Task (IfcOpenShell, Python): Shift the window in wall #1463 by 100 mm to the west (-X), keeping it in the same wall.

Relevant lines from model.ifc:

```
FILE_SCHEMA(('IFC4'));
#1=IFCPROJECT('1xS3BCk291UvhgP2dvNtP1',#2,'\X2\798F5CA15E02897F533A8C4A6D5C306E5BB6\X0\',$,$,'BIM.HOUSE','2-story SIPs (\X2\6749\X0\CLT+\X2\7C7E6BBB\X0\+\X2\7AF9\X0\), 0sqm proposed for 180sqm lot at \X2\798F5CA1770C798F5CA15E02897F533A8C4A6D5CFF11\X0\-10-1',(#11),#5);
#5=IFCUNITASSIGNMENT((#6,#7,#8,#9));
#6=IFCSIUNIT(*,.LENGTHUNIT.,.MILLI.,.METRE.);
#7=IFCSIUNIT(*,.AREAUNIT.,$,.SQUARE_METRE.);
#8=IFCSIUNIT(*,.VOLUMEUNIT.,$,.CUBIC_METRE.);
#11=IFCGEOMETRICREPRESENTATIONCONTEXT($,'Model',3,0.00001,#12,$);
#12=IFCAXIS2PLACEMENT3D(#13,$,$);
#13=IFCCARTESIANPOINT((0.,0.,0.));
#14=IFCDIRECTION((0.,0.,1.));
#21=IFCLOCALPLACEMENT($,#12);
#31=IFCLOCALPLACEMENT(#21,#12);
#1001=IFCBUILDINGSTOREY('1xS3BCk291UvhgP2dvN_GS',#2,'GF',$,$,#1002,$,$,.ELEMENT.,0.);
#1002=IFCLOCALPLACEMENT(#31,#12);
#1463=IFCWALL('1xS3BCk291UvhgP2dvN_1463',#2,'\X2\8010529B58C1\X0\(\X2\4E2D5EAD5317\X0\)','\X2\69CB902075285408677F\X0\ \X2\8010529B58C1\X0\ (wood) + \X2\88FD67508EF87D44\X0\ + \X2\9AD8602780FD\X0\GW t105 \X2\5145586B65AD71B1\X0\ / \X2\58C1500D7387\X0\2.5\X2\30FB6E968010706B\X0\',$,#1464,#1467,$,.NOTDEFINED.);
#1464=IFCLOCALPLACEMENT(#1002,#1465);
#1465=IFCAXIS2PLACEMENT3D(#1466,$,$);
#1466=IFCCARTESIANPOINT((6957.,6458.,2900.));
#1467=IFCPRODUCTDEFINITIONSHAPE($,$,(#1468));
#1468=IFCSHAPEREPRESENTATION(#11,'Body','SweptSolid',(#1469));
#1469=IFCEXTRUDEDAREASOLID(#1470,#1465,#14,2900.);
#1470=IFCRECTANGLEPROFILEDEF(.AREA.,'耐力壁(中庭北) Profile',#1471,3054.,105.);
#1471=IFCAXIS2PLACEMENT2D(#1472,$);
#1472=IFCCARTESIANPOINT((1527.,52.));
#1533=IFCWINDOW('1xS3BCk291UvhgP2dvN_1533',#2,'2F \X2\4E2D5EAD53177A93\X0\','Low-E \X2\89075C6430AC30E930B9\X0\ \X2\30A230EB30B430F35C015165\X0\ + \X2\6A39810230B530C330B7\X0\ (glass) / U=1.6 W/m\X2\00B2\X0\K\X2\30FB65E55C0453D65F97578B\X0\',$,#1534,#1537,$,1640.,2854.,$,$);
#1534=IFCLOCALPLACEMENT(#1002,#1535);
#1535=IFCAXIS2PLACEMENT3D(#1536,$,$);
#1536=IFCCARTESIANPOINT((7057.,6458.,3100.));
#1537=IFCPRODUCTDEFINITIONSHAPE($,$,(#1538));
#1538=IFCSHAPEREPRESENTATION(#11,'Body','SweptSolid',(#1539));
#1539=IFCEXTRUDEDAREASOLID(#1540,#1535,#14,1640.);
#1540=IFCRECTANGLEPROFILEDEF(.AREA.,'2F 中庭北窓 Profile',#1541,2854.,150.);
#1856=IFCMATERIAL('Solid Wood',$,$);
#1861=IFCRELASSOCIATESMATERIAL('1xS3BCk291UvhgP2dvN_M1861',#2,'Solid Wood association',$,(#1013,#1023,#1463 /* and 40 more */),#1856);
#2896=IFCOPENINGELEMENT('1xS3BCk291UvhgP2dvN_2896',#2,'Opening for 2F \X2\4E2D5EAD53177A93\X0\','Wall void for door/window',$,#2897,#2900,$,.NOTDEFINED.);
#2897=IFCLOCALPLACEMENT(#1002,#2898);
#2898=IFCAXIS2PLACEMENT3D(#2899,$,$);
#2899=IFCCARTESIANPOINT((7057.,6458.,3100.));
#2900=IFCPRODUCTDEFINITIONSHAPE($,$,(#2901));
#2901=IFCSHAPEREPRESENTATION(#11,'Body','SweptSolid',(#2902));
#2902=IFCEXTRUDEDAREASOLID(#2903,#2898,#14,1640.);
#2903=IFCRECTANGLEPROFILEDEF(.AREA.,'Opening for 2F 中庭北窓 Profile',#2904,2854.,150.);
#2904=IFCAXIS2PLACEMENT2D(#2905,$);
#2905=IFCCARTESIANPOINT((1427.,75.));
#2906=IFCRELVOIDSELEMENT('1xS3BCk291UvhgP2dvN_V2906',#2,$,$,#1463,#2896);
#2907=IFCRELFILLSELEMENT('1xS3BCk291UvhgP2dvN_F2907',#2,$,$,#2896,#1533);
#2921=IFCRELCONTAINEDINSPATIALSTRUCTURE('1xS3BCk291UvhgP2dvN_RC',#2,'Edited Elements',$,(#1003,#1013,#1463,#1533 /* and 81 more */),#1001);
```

```python
import ifcopenshell
import ifcopenshell.api.geometry
import ifcopenshell.util.placement
import ifcopenshell.util.unit

model = ifcopenshell.open("model.ifc")
unit_scale = ifcopenshell.util.unit.calculate_unit_scale(model)

window = model.by_id(1533)
opening = window.FillsVoids[0].RelatingOpeningElement
wall = opening.VoidsElements[0].RelatingBuildingElement

wall_matrix = ifcopenshell.util.placement.get_local_placement(wall.ObjectPlacement)
shift = wall_matrix[:3, 0] * -0.1 / unit_scale
before = ifcopenshell.util.placement.get_local_placement(window.ObjectPlacement)[:3, 3].copy()

# The window is not placed relative to its opening, so move both.
for product in (opening, window):
    matrix = ifcopenshell.util.placement.get_local_placement(product.ObjectPlacement)
    matrix[:3, 3] += shift
    ifcopenshell.api.geometry.edit_object_placement(model, product=product, matrix=matrix, is_si=False)

after = ifcopenshell.util.placement.get_local_placement(window.ObjectPlacement)[:3, 3]
print("window moved by", (after - before).round(3) + 0.0)

model.write("model_rev.ifc")
```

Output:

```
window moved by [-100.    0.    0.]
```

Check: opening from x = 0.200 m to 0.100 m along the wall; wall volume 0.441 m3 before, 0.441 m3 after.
